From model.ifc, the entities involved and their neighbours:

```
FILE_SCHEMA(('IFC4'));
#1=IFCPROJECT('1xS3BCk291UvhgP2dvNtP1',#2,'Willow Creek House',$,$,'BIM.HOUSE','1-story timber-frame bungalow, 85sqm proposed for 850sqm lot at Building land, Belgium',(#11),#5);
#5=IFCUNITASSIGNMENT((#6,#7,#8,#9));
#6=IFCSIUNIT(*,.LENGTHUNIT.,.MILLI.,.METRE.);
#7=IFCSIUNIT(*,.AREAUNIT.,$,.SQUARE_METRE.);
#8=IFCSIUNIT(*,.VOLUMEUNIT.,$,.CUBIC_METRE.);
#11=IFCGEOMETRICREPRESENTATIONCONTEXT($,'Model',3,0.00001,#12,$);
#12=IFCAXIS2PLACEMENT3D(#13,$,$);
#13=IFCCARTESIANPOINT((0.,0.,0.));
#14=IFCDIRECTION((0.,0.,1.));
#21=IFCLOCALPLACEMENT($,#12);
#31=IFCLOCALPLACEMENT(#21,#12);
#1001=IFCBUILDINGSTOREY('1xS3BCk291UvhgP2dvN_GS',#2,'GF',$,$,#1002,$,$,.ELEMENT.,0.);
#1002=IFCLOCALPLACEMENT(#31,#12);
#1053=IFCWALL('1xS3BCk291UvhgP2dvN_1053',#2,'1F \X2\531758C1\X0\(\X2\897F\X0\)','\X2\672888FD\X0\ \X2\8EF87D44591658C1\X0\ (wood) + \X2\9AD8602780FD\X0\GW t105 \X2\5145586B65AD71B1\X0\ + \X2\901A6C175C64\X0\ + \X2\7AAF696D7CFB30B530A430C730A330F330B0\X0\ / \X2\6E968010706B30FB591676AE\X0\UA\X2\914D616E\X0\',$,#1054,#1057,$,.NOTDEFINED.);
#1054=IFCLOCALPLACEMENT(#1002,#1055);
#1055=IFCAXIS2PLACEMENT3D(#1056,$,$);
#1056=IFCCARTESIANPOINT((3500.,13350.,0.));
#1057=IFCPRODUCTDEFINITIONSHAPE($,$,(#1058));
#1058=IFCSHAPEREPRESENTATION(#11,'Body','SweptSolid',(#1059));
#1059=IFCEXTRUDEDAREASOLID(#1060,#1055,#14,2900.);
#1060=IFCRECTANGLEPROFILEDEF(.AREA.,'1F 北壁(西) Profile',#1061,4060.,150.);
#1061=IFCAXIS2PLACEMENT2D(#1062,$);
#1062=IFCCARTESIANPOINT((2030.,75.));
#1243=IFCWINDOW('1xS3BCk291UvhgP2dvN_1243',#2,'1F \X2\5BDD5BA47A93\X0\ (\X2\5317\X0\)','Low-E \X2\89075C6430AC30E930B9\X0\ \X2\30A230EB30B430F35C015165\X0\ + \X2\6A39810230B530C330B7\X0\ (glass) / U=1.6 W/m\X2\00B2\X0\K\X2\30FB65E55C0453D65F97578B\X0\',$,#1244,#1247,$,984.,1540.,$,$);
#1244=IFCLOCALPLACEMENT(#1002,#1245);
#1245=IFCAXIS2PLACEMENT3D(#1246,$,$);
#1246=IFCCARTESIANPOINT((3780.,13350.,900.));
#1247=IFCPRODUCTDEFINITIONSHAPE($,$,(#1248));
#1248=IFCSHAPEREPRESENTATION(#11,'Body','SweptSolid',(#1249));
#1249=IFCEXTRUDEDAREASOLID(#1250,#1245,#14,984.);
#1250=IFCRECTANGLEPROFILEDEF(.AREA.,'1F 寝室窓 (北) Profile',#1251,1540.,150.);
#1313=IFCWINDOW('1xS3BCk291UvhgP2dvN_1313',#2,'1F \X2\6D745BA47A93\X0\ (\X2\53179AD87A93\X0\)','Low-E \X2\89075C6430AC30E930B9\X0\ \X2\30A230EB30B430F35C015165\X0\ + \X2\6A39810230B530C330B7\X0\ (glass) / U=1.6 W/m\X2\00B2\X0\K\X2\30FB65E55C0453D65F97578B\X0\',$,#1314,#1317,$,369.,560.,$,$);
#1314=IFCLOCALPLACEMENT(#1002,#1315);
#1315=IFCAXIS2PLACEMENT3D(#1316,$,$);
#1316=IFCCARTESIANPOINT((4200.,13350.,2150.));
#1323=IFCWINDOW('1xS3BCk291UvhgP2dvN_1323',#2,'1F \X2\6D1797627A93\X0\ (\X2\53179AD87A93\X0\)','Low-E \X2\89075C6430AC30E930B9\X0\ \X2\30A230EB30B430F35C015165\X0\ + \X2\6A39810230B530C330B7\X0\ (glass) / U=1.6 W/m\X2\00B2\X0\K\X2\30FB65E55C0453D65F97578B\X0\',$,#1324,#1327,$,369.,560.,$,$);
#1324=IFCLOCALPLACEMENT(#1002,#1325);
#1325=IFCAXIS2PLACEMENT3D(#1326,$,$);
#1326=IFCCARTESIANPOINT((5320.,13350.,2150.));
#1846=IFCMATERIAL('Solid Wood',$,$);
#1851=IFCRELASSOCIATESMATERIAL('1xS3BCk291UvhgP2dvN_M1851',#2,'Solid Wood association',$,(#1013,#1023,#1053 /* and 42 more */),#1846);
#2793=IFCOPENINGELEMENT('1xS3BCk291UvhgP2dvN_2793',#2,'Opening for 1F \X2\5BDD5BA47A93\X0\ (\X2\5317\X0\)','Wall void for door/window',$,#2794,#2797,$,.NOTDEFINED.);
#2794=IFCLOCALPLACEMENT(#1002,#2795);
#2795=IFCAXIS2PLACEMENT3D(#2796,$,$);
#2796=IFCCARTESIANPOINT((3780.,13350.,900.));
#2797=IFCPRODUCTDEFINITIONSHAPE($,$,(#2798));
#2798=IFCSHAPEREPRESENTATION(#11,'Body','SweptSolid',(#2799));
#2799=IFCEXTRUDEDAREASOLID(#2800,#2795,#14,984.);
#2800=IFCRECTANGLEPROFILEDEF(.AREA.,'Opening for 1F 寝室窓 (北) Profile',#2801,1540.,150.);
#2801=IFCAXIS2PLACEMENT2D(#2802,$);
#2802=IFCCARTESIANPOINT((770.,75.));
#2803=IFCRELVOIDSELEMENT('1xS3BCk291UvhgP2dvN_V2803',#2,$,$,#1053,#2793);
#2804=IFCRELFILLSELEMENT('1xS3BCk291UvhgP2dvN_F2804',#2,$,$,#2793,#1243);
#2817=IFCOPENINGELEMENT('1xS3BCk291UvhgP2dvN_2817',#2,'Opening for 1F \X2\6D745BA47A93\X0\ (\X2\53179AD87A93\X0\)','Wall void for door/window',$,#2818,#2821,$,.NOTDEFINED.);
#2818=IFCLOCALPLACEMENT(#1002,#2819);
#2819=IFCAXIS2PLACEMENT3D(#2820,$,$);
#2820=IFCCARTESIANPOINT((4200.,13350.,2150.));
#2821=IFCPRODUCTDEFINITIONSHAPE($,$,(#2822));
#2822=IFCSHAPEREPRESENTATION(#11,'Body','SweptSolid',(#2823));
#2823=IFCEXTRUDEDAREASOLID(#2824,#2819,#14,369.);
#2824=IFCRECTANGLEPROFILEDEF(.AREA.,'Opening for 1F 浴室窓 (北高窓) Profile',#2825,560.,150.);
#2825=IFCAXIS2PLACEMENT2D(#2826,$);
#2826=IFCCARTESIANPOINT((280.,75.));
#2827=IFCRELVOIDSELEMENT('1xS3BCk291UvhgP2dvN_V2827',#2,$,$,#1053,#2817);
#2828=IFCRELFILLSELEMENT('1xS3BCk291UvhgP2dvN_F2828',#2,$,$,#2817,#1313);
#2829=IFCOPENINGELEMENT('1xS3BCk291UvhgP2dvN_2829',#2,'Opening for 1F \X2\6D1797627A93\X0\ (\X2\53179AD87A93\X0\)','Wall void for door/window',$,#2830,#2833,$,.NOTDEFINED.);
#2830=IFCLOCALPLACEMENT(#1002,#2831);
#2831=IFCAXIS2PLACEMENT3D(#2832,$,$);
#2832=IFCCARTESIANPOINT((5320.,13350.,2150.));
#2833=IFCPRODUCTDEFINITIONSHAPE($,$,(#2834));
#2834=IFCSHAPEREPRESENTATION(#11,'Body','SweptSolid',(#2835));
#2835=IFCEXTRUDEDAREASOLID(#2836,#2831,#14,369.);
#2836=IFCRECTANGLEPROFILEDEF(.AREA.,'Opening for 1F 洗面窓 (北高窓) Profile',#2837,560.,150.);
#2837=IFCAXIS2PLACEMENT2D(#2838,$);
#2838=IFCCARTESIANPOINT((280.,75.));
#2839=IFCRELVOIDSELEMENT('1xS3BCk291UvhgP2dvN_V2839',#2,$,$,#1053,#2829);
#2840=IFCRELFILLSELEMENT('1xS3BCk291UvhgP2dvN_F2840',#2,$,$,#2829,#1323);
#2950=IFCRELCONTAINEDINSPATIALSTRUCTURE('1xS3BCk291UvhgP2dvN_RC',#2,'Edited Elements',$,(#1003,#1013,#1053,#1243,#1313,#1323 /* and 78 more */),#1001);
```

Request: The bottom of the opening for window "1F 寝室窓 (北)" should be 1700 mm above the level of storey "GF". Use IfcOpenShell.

```python
import numpy as np
import ifcopenshell
import ifcopenshell.api.geometry
import ifcopenshell.geom
import ifcopenshell.util.element
import ifcopenshell.util.placement
import ifcopenshell.util.shape
import ifcopenshell.util.unit

model = ifcopenshell.open("model.ifc")
unit_scale = ifcopenshell.util.unit.calculate_unit_scale(model)

window = model.by_guid("1xS3BCk291UvhgP2dvN_1243")
opening = window.FillsVoids[0].RelatingOpeningElement
storey = ifcopenshell.util.element.get_container(window, ifc_class="IfcBuildingStorey")
level = ifcopenshell.util.placement.get_local_placement(storey.ObjectPlacement)[2, 3]

# The opening's origin need not be at the sill, so measure its lowest point.
shape = ifcopenshell.geom.create_shape(ifcopenshell.geom.settings(), opening)
bottom = ifcopenshell.util.shape.get_shape_bottom_elevation(shape, shape.geometry) / unit_scale
dz = level + 1.7 / unit_scale - bottom

shift = np.array([0.0, 0.0, dz])
# The window is not placed relative to its opening, so move both.
for product in (opening, window):
    matrix = ifcopenshell.util.placement.get_local_placement(product.ObjectPlacement)
    matrix[:3, 3] += shift
    ifcopenshell.api.geometry.edit_object_placement(model, product=product, matrix=matrix, is_si=False)

print(f"moved by {dz * unit_scale:+.3f} m")

model.write("model_rev.ifc")
```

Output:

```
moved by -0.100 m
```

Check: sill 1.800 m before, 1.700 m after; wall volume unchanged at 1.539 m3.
